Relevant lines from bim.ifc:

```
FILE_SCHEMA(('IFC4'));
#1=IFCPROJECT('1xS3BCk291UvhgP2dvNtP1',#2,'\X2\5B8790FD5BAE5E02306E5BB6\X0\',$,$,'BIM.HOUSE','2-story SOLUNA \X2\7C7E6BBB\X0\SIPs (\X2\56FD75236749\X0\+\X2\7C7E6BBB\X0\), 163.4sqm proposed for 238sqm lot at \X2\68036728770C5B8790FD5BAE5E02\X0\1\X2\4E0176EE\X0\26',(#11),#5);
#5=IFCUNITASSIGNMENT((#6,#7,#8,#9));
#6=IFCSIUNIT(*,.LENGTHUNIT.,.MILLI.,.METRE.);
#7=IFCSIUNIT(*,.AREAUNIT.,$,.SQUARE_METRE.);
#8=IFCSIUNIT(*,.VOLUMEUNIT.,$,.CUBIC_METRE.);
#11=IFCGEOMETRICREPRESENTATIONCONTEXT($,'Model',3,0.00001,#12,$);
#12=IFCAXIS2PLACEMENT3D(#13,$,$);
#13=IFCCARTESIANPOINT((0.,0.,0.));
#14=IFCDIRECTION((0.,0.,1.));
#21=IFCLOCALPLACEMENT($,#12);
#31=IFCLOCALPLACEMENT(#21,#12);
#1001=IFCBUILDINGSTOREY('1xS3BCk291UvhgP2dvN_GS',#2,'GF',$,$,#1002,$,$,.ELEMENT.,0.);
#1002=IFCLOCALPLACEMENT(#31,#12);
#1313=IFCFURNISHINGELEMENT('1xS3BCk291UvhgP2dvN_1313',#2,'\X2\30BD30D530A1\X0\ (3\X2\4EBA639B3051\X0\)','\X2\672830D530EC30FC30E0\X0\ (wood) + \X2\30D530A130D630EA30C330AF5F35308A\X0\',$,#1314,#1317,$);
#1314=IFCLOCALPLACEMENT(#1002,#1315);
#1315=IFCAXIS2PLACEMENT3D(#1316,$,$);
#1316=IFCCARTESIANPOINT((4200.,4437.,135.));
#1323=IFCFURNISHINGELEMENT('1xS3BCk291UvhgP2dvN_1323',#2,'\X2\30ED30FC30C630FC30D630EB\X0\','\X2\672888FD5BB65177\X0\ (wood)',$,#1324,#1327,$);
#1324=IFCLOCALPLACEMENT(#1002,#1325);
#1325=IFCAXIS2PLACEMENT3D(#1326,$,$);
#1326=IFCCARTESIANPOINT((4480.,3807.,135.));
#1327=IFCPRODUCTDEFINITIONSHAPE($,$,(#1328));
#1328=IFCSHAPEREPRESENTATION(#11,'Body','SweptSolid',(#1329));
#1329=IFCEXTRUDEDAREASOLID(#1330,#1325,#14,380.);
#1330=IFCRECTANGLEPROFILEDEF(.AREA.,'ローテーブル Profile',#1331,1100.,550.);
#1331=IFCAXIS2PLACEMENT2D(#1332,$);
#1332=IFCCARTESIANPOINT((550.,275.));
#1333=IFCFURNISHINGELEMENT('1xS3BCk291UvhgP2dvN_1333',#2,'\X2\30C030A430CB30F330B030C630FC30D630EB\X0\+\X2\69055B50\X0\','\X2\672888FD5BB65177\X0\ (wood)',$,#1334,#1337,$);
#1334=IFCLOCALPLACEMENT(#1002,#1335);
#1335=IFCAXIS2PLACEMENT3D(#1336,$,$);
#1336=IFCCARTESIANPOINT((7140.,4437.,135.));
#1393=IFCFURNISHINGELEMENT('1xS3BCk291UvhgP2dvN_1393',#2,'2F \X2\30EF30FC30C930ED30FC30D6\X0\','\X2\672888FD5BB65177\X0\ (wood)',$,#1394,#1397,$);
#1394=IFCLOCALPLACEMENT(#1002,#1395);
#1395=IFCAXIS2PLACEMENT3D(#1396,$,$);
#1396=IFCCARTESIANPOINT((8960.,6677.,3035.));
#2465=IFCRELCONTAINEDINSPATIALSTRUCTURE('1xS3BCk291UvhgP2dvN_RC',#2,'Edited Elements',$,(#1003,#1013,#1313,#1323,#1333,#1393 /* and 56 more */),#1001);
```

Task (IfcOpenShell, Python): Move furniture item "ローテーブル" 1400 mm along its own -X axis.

```python
import ifcopenshell
import ifcopenshell.api.geometry
import ifcopenshell.util.placement
import ifcopenshell.util.unit

model = ifcopenshell.open("bim.ifc")
unit_scale = ifcopenshell.util.unit.calculate_unit_scale(model)

item = model.by_id(1323)
matrix = ifcopenshell.util.placement.get_local_placement(item.ObjectPlacement)
matrix[:3, 3] -= matrix[:3, 0] * 1.4 / unit_scale
ifcopenshell.api.geometry.edit_object_placement(model, product=item, matrix=matrix, is_si=False)

print(ifcopenshell.util.placement.get_local_placement(item.ObjectPlacement).round(3) + 0.0)

model.write("bim_v2.ifc")
```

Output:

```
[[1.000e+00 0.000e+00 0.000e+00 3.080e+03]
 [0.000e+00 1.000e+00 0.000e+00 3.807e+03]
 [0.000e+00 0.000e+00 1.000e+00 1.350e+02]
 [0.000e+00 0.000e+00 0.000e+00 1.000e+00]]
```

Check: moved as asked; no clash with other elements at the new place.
